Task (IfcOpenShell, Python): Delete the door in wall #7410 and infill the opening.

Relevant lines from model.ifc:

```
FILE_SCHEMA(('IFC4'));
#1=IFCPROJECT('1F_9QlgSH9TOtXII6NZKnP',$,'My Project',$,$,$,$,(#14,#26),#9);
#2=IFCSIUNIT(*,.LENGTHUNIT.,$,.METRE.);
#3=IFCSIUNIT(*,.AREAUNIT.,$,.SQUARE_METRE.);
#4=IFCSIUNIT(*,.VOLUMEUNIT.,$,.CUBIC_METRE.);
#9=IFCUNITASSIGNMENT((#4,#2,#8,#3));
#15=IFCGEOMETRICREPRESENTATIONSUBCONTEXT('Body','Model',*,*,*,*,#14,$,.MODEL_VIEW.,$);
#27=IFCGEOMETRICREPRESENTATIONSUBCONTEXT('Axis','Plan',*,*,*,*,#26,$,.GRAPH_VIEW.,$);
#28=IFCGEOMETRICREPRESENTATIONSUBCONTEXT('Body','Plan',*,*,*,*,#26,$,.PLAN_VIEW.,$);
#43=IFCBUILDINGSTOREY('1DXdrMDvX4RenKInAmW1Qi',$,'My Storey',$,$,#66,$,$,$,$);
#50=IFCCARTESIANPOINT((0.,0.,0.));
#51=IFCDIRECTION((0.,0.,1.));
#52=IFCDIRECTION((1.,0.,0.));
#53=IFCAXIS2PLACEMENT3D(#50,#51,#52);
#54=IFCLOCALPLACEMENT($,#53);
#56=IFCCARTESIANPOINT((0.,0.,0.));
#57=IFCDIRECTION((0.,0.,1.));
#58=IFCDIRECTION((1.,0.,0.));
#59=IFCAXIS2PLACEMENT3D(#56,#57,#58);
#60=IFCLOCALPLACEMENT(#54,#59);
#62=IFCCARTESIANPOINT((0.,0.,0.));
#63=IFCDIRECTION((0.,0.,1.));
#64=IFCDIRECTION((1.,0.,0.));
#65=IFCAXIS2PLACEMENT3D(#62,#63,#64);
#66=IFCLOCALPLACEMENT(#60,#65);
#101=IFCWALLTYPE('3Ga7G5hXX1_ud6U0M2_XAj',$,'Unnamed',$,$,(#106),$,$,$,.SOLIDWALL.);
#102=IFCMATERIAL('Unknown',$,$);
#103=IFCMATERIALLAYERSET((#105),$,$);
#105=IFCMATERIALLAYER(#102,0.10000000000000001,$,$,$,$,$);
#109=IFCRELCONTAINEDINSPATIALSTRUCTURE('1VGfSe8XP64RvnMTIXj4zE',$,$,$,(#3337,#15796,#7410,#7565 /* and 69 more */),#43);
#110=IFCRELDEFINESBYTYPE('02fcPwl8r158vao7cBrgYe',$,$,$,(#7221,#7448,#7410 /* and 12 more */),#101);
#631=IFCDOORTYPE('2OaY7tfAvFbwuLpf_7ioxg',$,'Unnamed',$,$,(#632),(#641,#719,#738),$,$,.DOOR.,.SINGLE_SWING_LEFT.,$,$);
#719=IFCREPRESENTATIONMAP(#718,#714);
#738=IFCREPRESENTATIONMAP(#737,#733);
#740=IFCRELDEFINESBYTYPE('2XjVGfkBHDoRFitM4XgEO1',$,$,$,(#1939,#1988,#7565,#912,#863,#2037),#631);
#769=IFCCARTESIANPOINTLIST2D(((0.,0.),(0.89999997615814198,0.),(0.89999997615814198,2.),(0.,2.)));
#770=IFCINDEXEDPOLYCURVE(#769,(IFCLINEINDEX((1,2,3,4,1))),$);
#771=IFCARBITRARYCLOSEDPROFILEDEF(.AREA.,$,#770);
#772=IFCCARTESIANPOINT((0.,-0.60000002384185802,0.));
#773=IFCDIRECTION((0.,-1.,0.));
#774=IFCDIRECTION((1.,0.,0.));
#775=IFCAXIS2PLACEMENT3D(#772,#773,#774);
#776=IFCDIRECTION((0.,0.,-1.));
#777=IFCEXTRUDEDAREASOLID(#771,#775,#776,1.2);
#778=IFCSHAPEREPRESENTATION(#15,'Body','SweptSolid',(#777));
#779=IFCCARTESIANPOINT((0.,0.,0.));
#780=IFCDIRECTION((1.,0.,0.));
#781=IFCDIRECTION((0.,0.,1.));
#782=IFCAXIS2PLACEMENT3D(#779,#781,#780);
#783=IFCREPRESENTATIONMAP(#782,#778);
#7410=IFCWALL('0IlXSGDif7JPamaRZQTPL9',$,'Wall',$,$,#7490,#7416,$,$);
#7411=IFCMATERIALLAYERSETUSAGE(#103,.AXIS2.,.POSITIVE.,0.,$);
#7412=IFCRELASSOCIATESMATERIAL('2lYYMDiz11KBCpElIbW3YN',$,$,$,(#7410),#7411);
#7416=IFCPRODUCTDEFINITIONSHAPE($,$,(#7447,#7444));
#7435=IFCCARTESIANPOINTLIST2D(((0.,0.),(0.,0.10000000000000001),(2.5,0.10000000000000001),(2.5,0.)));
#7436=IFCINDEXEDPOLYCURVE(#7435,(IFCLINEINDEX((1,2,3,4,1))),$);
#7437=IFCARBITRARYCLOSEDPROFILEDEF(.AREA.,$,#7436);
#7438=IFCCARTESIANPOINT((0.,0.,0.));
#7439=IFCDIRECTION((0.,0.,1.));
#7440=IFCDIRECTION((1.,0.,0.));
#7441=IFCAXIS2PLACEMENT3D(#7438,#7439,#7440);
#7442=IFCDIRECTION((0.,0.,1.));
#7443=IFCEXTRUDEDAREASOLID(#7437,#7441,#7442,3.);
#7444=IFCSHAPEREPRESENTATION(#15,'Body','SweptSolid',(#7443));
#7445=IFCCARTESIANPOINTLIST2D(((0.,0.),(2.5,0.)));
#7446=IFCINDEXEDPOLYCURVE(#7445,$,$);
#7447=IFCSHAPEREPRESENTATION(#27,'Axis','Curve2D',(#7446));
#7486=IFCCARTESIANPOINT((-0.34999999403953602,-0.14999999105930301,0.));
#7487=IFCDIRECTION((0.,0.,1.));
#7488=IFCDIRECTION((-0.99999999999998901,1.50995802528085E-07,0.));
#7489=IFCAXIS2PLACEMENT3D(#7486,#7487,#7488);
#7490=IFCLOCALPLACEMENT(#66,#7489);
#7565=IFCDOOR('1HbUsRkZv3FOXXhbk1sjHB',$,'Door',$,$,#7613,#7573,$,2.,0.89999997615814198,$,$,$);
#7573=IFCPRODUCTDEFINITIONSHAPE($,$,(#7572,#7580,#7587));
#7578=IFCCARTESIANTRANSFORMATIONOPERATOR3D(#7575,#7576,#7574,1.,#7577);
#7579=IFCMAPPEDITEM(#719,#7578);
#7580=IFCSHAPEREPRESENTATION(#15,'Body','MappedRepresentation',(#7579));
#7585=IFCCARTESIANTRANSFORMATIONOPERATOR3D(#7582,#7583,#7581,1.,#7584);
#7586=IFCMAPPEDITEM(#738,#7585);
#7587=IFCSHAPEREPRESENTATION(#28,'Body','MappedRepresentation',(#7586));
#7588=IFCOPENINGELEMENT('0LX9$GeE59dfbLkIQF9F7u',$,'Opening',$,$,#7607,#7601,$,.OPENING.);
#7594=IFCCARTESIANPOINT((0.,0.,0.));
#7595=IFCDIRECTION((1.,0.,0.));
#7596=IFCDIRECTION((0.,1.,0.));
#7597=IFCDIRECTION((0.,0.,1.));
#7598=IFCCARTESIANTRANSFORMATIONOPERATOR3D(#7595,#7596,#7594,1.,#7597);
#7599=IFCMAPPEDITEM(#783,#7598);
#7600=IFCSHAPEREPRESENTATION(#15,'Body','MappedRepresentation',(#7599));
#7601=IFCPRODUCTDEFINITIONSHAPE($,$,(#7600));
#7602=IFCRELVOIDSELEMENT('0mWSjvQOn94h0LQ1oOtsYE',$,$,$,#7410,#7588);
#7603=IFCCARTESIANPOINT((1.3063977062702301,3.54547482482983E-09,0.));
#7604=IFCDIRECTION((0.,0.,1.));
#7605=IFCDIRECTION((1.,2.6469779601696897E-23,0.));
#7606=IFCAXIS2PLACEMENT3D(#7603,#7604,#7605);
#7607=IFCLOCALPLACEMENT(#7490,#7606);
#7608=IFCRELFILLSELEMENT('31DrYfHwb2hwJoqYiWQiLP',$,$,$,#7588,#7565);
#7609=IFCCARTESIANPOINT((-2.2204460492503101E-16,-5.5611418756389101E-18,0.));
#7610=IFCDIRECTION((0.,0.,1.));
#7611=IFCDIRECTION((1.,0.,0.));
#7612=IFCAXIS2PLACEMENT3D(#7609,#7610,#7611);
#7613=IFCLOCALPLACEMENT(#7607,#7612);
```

```python
import ifcopenshell
import ifcopenshell.api.feature
import ifcopenshell.api.root
import ifcopenshell.geom
import ifcopenshell.util.shape

model = ifcopenshell.open("model.ifc")
settings = ifcopenshell.geom.settings()


def volume(element):
    """Net volume in cubic metres, openings subtracted."""
    shape = ifcopenshell.geom.create_shape(settings, element)
    return ifcopenshell.util.shape.get_volume(shape.geometry)


door = model.by_guid("1HbUsRkZv3FOXXhbk1sjHB")
opening = door.FillsVoids[0].RelatingOpeningElement
wall = opening.VoidsElements[0].RelatingBuildingElement
before = volume(wall)

ifcopenshell.api.root.remove_product(model, product=door)
ifcopenshell.api.feature.remove_feature(model, feature=opening)

after = volume(wall)

print(f"wall volume {before:.3f} -> {after:.3f} m3")

model.write("model-out.ifc")
```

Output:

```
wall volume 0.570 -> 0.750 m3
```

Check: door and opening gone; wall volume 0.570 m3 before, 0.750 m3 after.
